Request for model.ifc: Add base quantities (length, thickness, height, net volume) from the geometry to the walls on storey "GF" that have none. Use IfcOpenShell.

First a look at what the model holds.

```python
import ifcopenshell
import ifcopenshell.util.element
import ifcopenshell.util.unit

model = ifcopenshell.open("model.ifc")
print(model.schema)
for unit_type in ("LENGTHUNIT", "AREAUNIT", "VOLUMEUNIT"):
    print(unit_type, ifcopenshell.util.unit.calculate_unit_scale(model, unit_type))
storey = next(s for s in model.by_type("IfcBuildingStorey") if s.Name == "GF")
walls = [e for e in ifcopenshell.util.element.get_decomposition(storey) if e.is_a("IfcWall")]
for e in sorted(walls, key=lambda e: e.id()):
    print(e.id(), e.is_a(), e.Name, list(ifcopenshell.util.element.get_psets(e, qtos_only=True)), sep=" | ")
```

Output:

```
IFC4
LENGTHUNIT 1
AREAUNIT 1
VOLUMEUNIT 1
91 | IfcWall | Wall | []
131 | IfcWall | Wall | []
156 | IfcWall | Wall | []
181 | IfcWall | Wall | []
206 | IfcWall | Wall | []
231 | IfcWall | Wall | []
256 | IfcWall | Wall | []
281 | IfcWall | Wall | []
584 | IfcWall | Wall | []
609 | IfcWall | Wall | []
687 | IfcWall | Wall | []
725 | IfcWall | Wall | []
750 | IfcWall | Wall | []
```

```python
import ifcopenshell
import ifcopenshell.api.pset
import ifcopenshell.geom
import ifcopenshell.util.element
import ifcopenshell.util.shape
import ifcopenshell.util.unit

model = ifcopenshell.open("model.ifc")
unit_scale = ifcopenshell.util.unit.calculate_unit_scale(model)
volume_scale = ifcopenshell.util.unit.calculate_unit_scale(model, "VOLUMEUNIT")
settings = ifcopenshell.geom.settings()

storey = next(s for s in model.by_type("IfcBuildingStorey") if s.Name == "GF")
walls = [e for e in ifcopenshell.util.element.get_decomposition(storey) if e.is_a("IfcWall")]

for e in sorted(walls, key=lambda e: e.id()):
    if ifcopenshell.util.element.get_psets(e, qtos_only=True, should_inherit=False):
        continue
    # Geometry comes back in metres, in the element's own axes.
    shape = ifcopenshell.geom.create_shape(settings, e)
    values = {
        "Length": ifcopenshell.util.shape.get_x(shape.geometry) / unit_scale,
        "Width": ifcopenshell.util.shape.get_y(shape.geometry) / unit_scale,
        "Height": ifcopenshell.util.shape.get_z(shape.geometry) / unit_scale,
        "NetVolume": ifcopenshell.util.shape.get_volume(shape.geometry) / volume_scale,
    }
    qto = ifcopenshell.api.pset.add_qto(model, product=e, name="Qto_WallBaseQuantities")
    ifcopenshell.api.pset.edit_qto(model, qto=qto, properties=values)
    print(e.id(), {k: round(v, 3) for k, v in values.items()})

model.write("model_rev.ifc")
```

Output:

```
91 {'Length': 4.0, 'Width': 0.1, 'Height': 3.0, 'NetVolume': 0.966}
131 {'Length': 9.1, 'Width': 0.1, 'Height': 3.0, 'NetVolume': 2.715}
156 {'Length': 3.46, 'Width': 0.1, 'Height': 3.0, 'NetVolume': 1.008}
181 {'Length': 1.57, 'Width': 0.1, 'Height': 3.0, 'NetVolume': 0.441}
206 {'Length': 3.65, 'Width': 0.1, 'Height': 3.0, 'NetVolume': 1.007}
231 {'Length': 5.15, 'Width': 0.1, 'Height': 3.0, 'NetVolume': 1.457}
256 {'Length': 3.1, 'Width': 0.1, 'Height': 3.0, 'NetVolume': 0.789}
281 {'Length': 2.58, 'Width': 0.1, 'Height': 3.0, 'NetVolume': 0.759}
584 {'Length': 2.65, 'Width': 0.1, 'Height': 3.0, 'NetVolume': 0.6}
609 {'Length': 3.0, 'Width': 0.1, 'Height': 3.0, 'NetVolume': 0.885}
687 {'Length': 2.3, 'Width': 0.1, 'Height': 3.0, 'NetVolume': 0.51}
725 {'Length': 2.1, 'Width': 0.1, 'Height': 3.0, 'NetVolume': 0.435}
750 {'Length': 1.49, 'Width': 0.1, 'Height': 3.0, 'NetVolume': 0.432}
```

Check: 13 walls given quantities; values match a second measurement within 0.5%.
